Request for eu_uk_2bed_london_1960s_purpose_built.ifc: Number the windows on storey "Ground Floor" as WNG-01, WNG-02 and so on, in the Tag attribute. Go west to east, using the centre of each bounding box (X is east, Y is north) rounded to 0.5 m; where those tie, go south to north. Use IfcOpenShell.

First a look at what the model holds.

```python
import ifcopenshell
import ifcopenshell.util.element
import ifcopenshell.util.placement

model = ifcopenshell.open("eu_uk_2bed_london_1960s_purpose_built.ifc")
print(model.schema)
storey = next(s for s in model.by_type("IfcBuildingStorey") if s.Name == "Ground Floor")
windows = [e for e in ifcopenshell.util.element.get_decomposition(storey) if e.is_a("IfcWindow")]
for e in sorted(windows, key=lambda e: e.id()):
    origin = ifcopenshell.util.placement.get_local_placement(e.ObjectPlacement)[:3, 3]
    print(e.id(), e.Tag, e.Name, origin.round(2) + 0.0, sep=" | ")
```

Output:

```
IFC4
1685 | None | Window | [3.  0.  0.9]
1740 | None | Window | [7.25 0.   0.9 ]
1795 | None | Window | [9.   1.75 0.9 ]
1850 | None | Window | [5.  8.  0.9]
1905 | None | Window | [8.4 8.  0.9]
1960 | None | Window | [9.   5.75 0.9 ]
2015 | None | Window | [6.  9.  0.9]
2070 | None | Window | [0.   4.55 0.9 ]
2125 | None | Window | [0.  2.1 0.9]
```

```python
import ifcopenshell
import ifcopenshell.geom
import ifcopenshell.util.element
import ifcopenshell.util.shape

model = ifcopenshell.open("eu_uk_2bed_london_1960s_purpose_built.ifc")
settings = ifcopenshell.geom.settings()
settings.set("use-world-coords", True)


def centre(element):
    shape = ifcopenshell.geom.create_shape(settings, element)
    return ifcopenshell.util.shape.get_bbox_centroid(shape.geometry)


storey = next(s for s in model.by_type("IfcBuildingStorey") if s.Name == "Ground Floor")
windows = [e for e in ifcopenshell.util.element.get_decomposition(storey) if e.is_a("IfcWindow")]

# Insertion points can sit at a corner or the storey origin, so sort by the geometry (in metres).
centres = {e: centre(e) for e in windows}
windows.sort(key=lambda e: (round(centres[e][0] / 0.5), centres[e][1]))

for i, e in enumerate(windows, start=1):
    number = f"WNG-{i:02d}"
    e.Tag = number
    print(e.id(), number)

model.write("eu_uk_2bed_london_1960s_purpose_built_edited.ifc")
```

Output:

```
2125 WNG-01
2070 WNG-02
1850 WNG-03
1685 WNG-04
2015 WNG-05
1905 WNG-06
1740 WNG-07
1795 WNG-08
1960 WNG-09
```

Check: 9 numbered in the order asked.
